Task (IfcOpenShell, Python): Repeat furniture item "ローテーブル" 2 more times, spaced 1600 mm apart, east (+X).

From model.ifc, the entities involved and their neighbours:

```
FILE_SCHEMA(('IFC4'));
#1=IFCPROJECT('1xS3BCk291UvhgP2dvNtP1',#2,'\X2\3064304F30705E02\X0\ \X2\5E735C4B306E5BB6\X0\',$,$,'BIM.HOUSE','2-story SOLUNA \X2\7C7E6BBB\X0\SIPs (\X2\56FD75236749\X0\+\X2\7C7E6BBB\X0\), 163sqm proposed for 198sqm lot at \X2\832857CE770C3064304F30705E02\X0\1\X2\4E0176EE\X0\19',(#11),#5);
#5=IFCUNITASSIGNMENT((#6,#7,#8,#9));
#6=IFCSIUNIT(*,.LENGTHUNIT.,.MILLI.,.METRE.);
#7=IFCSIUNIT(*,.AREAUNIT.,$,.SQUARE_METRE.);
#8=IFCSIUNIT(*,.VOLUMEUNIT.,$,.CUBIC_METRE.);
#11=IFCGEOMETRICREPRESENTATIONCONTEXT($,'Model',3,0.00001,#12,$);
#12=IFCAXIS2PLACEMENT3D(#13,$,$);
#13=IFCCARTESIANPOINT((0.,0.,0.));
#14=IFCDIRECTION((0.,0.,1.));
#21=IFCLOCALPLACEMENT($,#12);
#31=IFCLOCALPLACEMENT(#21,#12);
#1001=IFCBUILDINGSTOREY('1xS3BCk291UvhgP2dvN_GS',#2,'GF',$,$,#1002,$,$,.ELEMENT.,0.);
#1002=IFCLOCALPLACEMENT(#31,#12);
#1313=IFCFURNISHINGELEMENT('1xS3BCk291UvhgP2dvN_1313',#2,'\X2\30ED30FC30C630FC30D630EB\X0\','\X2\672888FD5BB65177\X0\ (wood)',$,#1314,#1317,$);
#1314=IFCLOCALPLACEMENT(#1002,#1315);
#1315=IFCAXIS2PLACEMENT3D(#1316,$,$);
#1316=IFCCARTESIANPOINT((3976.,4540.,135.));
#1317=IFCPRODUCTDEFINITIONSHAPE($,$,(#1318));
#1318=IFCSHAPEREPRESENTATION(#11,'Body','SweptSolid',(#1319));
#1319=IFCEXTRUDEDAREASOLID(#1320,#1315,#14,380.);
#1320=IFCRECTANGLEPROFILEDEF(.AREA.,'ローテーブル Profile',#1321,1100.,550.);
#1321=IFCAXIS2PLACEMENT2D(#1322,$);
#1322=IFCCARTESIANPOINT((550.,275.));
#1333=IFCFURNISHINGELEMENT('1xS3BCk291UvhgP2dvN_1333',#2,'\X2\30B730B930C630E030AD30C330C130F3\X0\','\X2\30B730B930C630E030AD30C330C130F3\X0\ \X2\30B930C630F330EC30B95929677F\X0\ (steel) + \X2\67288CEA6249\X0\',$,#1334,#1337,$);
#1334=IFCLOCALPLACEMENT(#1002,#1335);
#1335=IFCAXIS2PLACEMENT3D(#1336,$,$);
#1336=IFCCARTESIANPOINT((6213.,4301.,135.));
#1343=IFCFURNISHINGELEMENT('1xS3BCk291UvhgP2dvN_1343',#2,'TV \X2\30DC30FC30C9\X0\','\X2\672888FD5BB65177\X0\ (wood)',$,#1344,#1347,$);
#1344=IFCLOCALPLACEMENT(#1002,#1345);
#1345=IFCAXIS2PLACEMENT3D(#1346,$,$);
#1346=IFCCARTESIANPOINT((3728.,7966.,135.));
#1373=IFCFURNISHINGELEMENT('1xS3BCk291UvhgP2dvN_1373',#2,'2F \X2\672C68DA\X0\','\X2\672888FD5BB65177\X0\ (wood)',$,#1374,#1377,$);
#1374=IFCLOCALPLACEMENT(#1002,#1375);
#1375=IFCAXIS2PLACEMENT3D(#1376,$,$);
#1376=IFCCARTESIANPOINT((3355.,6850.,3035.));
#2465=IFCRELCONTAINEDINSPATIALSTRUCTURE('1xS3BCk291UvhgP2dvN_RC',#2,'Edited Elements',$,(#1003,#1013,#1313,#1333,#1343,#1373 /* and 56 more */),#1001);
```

```python
import numpy as np
import ifcopenshell
import ifcopenshell.api.geometry
import ifcopenshell.api.root
import ifcopenshell.util.element
import ifcopenshell.util.placement
import ifcopenshell.util.unit

model = ifcopenshell.open("model.ifc")
unit_scale = ifcopenshell.util.unit.calculate_unit_scale(model)


def reuse_history(source, copy):
    """copy_class also copies each property set's owner history, people and application; keep the originals."""
    for rel in copy.IsDefinedBy:
        if rel.is_a("IfcRelDefinesByProperties") and (history := rel.RelatingPropertyDefinition.OwnerHistory):
            rel.RelatingPropertyDefinition.OwnerHistory = source.OwnerHistory
            ifcopenshell.util.element.remove_deep2(model, history)


source = model.by_guid("1xS3BCk291UvhgP2dvN_1313")
base = ifcopenshell.util.placement.get_local_placement(source.ObjectPlacement)
step = np.array([1.0, 0.0, 0.0]) * 1.6 / unit_scale

for i in range(1, 3):
    copy = ifcopenshell.api.root.copy_class(model, product=source)
    copy.Representation = ifcopenshell.util.element.copy_deep(
        model, source.Representation, exclude=["IfcGeometricRepresentationContext", "IfcRepresentationMap"]
    )
    reuse_history(source, copy)
    matrix = base.copy()
    matrix[:3, 3] += i * step
    print("added at", matrix[:3, 3].round(3) + 0.0)
    ifcopenshell.api.geometry.edit_object_placement(model, product=copy, matrix=matrix, is_si=False)

model.write("model-out.ifc")
```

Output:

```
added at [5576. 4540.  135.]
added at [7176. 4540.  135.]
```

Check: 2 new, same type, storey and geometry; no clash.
